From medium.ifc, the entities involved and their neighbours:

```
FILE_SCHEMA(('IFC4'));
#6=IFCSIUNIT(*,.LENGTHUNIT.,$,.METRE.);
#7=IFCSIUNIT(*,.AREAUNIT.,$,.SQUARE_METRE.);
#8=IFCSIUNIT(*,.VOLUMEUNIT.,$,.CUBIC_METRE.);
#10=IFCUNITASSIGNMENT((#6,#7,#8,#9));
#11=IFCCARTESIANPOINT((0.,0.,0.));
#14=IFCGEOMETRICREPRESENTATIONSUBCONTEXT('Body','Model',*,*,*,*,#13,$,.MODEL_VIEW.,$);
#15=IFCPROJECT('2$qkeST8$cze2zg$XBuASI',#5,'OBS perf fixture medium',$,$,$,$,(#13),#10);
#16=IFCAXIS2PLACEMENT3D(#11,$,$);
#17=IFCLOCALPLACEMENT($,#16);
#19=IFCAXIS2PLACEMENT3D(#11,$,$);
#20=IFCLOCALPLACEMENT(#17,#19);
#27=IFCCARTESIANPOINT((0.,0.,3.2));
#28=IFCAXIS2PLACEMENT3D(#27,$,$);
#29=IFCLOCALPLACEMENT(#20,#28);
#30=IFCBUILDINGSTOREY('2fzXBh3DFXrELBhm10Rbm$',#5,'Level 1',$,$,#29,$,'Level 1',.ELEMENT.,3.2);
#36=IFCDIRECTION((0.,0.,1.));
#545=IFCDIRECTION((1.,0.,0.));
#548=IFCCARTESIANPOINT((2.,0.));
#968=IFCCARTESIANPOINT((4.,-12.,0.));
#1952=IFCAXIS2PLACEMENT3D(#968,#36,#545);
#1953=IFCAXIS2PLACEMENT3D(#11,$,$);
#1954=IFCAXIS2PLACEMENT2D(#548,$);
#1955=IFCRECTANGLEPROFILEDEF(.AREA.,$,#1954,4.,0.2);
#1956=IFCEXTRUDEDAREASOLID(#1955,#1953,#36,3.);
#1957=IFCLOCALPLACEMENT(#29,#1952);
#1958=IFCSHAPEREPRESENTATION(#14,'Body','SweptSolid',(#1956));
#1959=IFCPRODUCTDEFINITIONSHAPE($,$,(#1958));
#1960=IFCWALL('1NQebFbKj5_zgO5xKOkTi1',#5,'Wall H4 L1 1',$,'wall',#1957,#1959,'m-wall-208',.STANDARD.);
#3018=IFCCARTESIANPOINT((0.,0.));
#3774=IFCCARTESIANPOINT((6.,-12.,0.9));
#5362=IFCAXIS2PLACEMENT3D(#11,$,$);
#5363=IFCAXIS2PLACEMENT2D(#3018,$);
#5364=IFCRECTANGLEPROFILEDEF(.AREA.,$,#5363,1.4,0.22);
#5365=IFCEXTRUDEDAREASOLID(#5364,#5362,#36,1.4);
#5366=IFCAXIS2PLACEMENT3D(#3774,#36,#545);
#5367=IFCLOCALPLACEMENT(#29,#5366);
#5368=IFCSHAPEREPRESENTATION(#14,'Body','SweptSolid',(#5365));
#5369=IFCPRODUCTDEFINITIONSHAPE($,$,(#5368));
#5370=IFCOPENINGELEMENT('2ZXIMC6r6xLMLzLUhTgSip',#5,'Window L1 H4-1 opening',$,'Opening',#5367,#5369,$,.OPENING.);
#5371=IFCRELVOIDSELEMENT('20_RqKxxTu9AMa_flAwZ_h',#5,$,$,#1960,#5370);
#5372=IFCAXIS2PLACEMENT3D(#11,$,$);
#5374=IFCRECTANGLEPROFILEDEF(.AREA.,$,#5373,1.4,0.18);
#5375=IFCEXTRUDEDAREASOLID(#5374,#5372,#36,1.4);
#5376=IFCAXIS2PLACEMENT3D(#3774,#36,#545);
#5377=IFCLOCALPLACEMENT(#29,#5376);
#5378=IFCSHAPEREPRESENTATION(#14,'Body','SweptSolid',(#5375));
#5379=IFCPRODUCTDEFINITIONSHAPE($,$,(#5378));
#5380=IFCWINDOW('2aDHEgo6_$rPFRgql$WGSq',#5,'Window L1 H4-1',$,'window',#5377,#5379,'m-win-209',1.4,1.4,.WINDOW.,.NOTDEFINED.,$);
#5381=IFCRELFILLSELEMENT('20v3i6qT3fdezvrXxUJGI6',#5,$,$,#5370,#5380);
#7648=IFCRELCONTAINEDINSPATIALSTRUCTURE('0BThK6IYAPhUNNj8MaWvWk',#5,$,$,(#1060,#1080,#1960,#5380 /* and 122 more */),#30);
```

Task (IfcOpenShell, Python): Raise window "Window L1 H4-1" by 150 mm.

```python
import numpy as np
import ifcopenshell
import ifcopenshell.api.geometry
import ifcopenshell.util.placement
import ifcopenshell.util.unit

model = ifcopenshell.open("medium.ifc")
unit_scale = ifcopenshell.util.unit.calculate_unit_scale(model)

window = model.by_guid("2aDHEgo6_$rPFRgql$WGSq")
opening = window.FillsVoids[0].RelatingOpeningElement
dz = 0.15 / unit_scale

shift = np.array([0.0, 0.0, dz])
# The window is not placed relative to its opening, so move both.
for product in (opening, window):
    matrix = ifcopenshell.util.placement.get_local_placement(product.ObjectPlacement)
    matrix[:3, 3] += shift
    ifcopenshell.api.geometry.edit_object_placement(model, product=product, matrix=matrix, is_si=False)

print(f"moved by {dz * unit_scale:+.3f} m")

model.write("medium_edited.ifc")
```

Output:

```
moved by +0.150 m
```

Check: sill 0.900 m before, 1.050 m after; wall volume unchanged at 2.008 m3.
